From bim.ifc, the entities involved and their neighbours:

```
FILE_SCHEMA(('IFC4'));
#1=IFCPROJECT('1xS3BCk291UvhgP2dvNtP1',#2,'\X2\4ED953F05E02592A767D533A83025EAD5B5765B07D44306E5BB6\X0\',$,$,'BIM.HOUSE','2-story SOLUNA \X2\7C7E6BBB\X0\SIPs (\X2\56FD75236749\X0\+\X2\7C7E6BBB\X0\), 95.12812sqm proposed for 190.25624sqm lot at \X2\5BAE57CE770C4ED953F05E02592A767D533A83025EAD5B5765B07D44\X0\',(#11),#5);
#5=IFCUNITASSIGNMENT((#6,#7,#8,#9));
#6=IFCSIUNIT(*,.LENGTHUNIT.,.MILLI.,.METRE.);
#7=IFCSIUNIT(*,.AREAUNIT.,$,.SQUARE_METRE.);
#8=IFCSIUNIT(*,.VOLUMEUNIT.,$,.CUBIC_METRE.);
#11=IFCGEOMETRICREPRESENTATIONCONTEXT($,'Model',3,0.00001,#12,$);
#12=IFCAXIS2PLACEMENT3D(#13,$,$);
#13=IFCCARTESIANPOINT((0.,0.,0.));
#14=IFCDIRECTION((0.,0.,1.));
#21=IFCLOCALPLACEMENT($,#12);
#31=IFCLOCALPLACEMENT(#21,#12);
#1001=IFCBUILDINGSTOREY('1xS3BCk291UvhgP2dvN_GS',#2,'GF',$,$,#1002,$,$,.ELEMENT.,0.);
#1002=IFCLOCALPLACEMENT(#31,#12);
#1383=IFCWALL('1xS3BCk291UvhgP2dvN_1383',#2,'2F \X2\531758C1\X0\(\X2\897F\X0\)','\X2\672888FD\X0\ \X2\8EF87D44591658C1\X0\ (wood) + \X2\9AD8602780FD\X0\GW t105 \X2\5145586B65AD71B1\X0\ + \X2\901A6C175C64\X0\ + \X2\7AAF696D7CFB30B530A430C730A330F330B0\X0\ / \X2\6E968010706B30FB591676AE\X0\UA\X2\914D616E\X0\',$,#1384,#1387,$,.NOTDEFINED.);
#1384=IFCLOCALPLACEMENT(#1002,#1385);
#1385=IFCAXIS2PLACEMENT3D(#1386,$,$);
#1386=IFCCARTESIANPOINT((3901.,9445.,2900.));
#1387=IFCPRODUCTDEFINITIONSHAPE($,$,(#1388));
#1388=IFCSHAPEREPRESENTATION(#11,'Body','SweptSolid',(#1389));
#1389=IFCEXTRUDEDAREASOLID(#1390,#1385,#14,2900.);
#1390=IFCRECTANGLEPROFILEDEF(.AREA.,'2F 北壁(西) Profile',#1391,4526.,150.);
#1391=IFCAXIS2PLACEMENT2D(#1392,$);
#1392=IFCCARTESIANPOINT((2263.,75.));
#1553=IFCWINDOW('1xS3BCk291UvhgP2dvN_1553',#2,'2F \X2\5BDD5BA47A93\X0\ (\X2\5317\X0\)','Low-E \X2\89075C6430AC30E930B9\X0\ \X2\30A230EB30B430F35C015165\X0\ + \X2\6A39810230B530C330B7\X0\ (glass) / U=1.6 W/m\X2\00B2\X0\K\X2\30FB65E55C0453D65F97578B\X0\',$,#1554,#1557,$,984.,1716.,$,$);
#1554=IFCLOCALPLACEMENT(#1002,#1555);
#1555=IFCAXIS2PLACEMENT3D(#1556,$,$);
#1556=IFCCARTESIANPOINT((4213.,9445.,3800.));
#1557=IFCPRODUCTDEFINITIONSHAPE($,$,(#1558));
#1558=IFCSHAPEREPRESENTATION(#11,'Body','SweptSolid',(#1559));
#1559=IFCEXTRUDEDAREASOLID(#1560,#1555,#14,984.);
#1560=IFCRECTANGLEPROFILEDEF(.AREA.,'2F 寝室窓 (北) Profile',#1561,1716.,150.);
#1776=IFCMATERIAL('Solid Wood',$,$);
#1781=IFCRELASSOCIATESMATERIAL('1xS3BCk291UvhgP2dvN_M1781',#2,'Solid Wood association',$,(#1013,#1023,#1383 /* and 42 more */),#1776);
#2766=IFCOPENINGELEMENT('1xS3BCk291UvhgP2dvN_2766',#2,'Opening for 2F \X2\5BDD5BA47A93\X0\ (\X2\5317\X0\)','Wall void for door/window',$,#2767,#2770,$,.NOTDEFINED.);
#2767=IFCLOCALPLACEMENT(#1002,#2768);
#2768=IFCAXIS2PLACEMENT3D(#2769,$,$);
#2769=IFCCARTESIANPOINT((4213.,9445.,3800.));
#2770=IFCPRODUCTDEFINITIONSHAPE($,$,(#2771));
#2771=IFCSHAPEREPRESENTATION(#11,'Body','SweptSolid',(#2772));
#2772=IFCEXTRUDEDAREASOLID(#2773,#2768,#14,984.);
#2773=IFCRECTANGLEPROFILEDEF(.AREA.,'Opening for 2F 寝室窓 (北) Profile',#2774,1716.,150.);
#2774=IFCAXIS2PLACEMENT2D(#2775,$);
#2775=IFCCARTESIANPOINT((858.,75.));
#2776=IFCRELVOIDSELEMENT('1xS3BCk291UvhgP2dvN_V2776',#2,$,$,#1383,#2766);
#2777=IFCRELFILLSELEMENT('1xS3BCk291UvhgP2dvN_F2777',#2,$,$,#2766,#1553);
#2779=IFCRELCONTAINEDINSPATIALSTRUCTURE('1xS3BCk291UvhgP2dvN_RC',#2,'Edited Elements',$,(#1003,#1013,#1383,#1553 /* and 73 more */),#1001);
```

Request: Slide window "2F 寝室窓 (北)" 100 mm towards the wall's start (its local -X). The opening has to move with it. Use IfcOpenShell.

```python
import ifcopenshell
import ifcopenshell.api.geometry
import ifcopenshell.util.placement

model = ifcopenshell.open("bim.ifc")

window = model.by_id(1553)
opening = window.FillsVoids[0].RelatingOpeningElement
wall = opening.VoidsElements[0].RelatingBuildingElement

wall_matrix = ifcopenshell.util.placement.get_local_placement(wall.ObjectPlacement)
shift = wall_matrix[:3, 0] * -100.0
before = ifcopenshell.util.placement.get_local_placement(window.ObjectPlacement)[:3, 3].copy()

# The window is not placed relative to its opening, so move both.
for product in (opening, window):
    matrix = ifcopenshell.util.placement.get_local_placement(product.ObjectPlacement)
    matrix[:3, 3] += shift
    ifcopenshell.api.geometry.edit_object_placement(model, product=product, matrix=matrix, is_si=False)

after = ifcopenshell.util.placement.get_local_placement(window.ObjectPlacement)[:3, 3]
print("window moved by", (after - before).round(3) + 0.0)

model.write("bim_edited.ifc")
```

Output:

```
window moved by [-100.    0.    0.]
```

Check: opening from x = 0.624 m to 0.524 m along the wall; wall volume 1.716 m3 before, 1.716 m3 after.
